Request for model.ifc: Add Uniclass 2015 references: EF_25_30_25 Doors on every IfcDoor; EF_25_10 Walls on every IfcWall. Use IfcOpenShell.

First a look at what the model holds.

```python
import ifcopenshell

model = ifcopenshell.open("model.ifc")
print(model.schema)
print("classifications:", [c.Name for c in model.by_type("IfcClassification")])
for ifc_class in ("IfcDoor", "IfcRoof", "IfcStair", "IfcWall", "IfcWindow"):
    print(ifc_class, len(model.by_type(ifc_class)))
```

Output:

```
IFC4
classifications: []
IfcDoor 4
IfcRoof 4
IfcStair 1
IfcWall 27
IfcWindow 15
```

```python
import ifcopenshell
import ifcopenshell.api.classification

model = ifcopenshell.open("model.ifc")

system = ifcopenshell.api.classification.add_classification(model, classification="Uniclass 2015")

codes = {
    "IfcDoor": ("EF_25_30_25", "Doors"),
    "IfcWall": ("EF_25_10", "Walls"),
}
for ifc_class, (code, name) in codes.items():
    products = model.by_type(ifc_class)
    ifcopenshell.api.classification.add_reference(
        model, products=products, classification=system, identification=code, name=name
    )
    print(code, len(products))

model.write("model_v2.ifc")
```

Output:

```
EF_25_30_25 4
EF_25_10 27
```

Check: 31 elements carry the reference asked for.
